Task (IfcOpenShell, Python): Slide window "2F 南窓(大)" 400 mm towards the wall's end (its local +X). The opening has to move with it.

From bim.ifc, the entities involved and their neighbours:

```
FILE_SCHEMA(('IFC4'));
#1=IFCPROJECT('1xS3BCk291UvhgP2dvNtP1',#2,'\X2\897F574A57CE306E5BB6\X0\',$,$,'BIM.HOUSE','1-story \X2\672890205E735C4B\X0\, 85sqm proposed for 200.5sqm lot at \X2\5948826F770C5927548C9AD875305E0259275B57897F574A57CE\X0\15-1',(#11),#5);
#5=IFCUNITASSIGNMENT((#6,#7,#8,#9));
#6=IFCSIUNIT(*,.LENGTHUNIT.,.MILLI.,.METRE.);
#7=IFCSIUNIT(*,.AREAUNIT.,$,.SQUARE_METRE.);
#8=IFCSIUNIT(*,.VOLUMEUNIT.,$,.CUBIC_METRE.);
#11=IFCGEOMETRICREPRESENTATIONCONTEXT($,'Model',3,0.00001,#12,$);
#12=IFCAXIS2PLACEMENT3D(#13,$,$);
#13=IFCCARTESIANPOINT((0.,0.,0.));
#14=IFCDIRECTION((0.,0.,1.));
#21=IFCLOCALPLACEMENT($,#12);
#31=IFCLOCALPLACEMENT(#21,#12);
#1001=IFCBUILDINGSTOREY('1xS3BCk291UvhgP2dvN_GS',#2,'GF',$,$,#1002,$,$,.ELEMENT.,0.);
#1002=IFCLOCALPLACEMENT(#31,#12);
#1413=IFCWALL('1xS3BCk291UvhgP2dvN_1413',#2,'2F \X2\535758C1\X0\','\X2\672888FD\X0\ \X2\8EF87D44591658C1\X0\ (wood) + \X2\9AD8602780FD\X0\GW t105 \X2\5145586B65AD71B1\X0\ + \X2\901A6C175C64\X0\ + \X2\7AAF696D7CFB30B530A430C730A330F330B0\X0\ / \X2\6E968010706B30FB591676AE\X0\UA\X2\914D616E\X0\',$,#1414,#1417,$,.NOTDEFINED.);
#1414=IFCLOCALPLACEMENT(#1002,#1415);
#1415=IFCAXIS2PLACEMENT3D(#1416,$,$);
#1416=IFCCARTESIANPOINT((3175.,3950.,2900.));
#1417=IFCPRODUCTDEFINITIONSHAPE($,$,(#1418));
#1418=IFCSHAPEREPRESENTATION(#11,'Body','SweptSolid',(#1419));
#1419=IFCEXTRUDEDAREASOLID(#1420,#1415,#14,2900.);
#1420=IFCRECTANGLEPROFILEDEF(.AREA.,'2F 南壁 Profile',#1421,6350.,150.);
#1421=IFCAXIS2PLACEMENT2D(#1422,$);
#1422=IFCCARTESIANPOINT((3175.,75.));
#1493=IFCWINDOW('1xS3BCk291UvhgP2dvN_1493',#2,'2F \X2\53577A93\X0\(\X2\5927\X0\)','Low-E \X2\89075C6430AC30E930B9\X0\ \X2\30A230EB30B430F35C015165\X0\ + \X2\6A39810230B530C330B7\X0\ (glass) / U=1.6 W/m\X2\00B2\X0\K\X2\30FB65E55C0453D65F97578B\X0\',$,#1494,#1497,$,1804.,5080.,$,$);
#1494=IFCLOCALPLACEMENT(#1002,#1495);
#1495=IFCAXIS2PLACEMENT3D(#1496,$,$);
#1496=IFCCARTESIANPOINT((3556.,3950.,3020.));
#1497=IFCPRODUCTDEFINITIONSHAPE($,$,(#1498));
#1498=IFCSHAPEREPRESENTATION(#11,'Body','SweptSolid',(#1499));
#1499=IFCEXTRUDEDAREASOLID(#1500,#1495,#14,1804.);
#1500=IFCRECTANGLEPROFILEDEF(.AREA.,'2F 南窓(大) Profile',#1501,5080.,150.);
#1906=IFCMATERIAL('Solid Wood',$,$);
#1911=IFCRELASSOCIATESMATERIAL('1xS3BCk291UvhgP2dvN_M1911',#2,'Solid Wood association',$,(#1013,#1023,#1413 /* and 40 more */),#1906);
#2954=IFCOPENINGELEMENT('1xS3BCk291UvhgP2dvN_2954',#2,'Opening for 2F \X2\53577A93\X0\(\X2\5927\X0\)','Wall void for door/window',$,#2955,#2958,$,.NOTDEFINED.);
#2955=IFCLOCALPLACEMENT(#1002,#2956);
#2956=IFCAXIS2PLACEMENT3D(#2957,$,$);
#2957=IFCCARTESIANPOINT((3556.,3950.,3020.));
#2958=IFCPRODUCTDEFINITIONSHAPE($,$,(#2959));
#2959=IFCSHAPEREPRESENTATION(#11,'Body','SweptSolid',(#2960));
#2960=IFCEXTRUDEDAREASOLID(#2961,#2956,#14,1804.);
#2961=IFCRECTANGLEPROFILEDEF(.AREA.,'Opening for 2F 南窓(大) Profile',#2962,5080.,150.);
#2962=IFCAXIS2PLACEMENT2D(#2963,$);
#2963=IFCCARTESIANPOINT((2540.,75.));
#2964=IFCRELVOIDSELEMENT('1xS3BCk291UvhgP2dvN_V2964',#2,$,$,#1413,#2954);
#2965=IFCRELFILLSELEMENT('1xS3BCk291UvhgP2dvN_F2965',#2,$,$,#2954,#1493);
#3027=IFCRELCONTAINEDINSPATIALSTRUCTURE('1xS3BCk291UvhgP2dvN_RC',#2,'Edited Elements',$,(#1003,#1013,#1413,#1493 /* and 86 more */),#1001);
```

```python
import ifcopenshell
import ifcopenshell.api.geometry
import ifcopenshell.util.placement
import ifcopenshell.util.unit

model = ifcopenshell.open("bim.ifc")
unit_scale = ifcopenshell.util.unit.calculate_unit_scale(model)

window = model.by_guid("1xS3BCk291UvhgP2dvN_1493")
opening = window.FillsVoids[0].RelatingOpeningElement
wall = opening.VoidsElements[0].RelatingBuildingElement

wall_matrix = ifcopenshell.util.placement.get_local_placement(wall.ObjectPlacement)
shift = wall_matrix[:3, 0] * 0.4 / unit_scale
before = ifcopenshell.util.placement.get_local_placement(window.ObjectPlacement)[:3, 3].copy()

# The window is not placed relative to its opening, so move both.
for product in (opening, window):
    matrix = ifcopenshell.util.placement.get_local_placement(product.ObjectPlacement)
    matrix[:3, 3] += shift
    ifcopenshell.api.geometry.edit_object_placement(model, product=product, matrix=matrix, is_si=False)

after = ifcopenshell.util.placement.get_local_placement(window.ObjectPlacement)[:3, 3]
print("window moved by", (after - before).round(3) + 0.0)

model.write("bim_updated.ifc")
```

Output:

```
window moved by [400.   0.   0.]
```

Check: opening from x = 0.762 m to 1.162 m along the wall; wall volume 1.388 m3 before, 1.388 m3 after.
